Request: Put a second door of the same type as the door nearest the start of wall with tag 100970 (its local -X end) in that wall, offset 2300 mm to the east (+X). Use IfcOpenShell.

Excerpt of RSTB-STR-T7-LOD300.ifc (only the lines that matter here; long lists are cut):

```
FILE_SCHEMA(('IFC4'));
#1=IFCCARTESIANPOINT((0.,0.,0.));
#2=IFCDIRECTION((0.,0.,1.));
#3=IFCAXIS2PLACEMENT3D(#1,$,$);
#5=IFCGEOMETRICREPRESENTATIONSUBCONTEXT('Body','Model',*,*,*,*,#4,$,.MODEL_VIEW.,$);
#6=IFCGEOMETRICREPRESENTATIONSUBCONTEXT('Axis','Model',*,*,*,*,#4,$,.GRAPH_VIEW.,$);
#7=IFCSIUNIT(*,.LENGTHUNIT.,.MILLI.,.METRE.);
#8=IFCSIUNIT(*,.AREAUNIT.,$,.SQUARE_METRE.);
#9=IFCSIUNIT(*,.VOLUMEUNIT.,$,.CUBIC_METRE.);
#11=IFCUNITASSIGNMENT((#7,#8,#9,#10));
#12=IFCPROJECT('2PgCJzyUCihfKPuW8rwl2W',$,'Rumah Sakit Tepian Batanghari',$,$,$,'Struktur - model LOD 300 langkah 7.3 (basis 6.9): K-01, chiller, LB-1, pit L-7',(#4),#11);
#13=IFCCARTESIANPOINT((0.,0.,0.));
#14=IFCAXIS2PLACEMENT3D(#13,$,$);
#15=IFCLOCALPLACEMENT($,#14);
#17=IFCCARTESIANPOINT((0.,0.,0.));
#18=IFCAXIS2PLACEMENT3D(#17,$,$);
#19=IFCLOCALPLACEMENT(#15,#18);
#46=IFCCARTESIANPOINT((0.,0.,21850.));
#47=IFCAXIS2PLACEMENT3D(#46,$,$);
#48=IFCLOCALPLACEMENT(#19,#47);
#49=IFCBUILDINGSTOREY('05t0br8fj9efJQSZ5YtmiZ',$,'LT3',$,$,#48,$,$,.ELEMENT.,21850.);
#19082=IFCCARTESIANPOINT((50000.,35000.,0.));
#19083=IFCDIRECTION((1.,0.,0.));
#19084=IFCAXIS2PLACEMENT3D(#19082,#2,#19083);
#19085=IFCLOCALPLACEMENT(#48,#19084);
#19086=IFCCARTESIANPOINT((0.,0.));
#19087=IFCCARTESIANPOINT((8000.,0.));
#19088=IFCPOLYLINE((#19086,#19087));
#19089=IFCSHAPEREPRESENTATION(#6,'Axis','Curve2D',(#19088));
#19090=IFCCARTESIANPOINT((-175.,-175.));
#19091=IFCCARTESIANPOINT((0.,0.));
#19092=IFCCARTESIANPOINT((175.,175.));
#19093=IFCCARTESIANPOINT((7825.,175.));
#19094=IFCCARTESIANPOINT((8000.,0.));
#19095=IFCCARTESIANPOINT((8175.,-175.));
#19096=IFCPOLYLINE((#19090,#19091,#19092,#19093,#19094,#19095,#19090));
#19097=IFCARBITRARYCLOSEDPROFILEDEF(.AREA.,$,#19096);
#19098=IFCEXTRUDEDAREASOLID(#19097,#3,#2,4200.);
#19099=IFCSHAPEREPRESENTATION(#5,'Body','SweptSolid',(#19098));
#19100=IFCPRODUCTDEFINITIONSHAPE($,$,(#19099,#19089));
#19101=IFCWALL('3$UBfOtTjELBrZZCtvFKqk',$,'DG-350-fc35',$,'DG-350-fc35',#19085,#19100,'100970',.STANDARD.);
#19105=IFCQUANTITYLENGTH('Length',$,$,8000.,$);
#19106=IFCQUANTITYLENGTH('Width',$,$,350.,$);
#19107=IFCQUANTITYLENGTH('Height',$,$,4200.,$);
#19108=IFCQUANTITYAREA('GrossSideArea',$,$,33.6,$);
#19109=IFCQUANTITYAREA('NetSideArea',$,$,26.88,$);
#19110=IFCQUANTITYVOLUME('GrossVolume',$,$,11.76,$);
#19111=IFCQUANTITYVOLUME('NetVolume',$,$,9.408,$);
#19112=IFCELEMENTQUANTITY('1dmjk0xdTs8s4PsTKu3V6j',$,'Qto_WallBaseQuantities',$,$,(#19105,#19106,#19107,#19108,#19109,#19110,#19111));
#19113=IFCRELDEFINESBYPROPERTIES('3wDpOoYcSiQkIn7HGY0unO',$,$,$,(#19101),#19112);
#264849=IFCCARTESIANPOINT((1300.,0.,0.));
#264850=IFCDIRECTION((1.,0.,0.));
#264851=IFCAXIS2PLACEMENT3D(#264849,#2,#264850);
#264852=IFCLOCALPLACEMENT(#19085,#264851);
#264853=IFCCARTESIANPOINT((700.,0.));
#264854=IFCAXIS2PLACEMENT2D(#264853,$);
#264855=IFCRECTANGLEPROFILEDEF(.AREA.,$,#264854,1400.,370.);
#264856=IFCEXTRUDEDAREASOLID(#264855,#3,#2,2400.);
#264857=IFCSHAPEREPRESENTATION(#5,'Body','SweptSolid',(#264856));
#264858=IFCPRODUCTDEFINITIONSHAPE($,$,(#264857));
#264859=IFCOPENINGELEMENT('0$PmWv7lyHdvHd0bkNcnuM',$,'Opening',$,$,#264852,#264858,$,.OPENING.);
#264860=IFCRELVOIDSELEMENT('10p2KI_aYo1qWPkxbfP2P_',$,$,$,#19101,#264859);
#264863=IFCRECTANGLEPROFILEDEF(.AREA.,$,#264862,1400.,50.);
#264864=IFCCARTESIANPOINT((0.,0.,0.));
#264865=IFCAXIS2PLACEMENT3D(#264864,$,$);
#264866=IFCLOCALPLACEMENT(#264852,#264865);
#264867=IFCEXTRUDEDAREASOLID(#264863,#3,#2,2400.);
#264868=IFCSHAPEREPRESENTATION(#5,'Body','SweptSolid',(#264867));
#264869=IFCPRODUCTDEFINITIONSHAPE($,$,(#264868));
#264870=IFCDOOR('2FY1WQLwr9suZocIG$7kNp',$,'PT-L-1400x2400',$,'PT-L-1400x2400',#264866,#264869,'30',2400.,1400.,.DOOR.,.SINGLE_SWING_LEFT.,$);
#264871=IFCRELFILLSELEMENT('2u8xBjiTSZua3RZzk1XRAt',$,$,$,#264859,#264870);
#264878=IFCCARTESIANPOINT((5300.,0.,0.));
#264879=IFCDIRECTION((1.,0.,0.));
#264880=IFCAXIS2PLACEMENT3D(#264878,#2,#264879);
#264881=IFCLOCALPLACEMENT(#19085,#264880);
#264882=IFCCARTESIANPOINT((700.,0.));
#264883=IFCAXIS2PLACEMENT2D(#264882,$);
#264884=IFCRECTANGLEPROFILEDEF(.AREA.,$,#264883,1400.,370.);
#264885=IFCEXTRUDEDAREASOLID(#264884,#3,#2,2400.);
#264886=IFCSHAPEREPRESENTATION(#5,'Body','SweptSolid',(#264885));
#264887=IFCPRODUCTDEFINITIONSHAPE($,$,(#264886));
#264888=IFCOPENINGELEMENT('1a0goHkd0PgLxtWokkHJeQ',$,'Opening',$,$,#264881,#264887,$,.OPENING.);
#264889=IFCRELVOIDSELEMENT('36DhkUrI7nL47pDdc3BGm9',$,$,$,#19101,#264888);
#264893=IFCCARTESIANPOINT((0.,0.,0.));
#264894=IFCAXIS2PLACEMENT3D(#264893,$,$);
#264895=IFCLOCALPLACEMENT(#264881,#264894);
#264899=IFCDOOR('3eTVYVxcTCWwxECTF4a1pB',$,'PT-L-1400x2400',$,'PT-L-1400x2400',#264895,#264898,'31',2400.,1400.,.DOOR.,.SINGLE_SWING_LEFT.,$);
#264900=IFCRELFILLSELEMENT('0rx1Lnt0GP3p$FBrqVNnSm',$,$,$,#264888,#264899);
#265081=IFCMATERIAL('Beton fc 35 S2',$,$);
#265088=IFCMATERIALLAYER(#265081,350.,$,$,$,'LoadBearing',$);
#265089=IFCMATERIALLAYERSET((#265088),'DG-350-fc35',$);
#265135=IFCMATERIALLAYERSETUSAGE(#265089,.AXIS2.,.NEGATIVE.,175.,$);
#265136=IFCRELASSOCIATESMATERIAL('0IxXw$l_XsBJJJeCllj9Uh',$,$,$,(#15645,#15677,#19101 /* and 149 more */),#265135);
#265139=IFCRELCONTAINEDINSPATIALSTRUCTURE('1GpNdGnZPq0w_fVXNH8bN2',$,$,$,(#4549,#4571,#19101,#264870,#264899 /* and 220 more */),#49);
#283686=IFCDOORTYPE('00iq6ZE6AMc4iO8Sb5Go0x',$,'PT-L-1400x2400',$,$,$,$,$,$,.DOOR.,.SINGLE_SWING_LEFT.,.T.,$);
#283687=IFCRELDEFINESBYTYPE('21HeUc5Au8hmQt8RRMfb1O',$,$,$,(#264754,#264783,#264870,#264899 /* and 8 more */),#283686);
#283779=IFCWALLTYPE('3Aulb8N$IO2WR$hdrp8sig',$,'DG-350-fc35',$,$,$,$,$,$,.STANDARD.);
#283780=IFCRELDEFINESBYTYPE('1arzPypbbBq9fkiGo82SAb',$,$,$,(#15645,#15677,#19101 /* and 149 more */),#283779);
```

```python
import ifcopenshell
import ifcopenshell.api.feature
import ifcopenshell.api.geometry
import ifcopenshell.api.pset
import ifcopenshell.api.root
import ifcopenshell.geom
import ifcopenshell.util.element
import ifcopenshell.util.placement
import ifcopenshell.util.shape
import ifcopenshell.util.unit

model = ifcopenshell.open("RSTB-STR-T7-LOD300.ifc")
unit_scale = ifcopenshell.util.unit.calculate_unit_scale(model)
area_scale = ifcopenshell.util.unit.calculate_unit_scale(model, "AREAUNIT")
volume_scale = ifcopenshell.util.unit.calculate_unit_scale(model, "VOLUMEUNIT")
settings = ifcopenshell.geom.settings()


def volume(element):
    """Net volume in cubic metres, openings subtracted."""
    shape = ifcopenshell.geom.create_shape(settings, element)
    return ifcopenshell.util.shape.get_volume(shape.geometry)


door = model.by_guid("2FY1WQLwr9suZocIG$7kNp")
opening = door.FillsVoids[0].RelatingOpeningElement
wall = opening.VoidsElements[0].RelatingBuildingElement
before = volume(wall)
shift = ifcopenshell.util.placement.get_local_placement(wall.ObjectPlacement)[:3, 0] * 2.3 / unit_scale

# copy_class copies the void relationship, type, container and properties, but no geometry.
new_opening = ifcopenshell.api.root.copy_class(model, product=opening)
new_opening.Representation = ifcopenshell.util.element.copy_deep(
    model, opening.Representation, exclude=["IfcGeometricRepresentationContext", "IfcRepresentationMap"]
)
new_door = ifcopenshell.api.root.copy_class(model, product=door)
new_door.Representation = ifcopenshell.util.element.copy_deep(
    model, door.Representation, exclude=["IfcGeometricRepresentationContext", "IfcRepresentationMap"]
)
new_door.Tag = None
ifcopenshell.api.feature.add_filling(model, opening=new_opening, element=new_door)

for old, new in ((opening, new_opening), (door, new_door)):
    matrix = ifcopenshell.util.placement.get_local_placement(old.ObjectPlacement)
    matrix[:3, 3] += shift
    ifcopenshell.api.geometry.edit_object_placement(model, product=new, matrix=matrix, is_si=False)

after = volume(wall)
thickness = 0.35  # wall thickness in metres

# Update the wall's stored quantities.
qto = model.by_id(ifcopenshell.util.element.get_pset(wall, "Qto_WallBaseQuantities", should_inherit=False)["id"])
ifcopenshell.api.pset.edit_qto(model, qto=qto, properties={
    "NetSideArea": after / thickness / area_scale,
    "NetVolume": after / volume_scale,
})

print(f"wall volume {before:.3f} -> {after:.3f} m3")

model.write("RSTB-STR-T7-LOD300_edited.ifc")
```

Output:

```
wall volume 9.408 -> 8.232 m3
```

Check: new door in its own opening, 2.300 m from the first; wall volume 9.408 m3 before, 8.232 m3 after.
